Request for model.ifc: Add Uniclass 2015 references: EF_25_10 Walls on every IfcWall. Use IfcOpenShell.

First a look at what the model holds.

```python
import ifcopenshell

model = ifcopenshell.open("model.ifc")
print(model.schema)
print("classifications:", [c.Name for c in model.by_type("IfcClassification")])
for ifc_class in ("IfcDoor", "IfcRoof", "IfcStair", "IfcWall", "IfcWindow"):
    print(ifc_class, len(model.by_type(ifc_class)))
```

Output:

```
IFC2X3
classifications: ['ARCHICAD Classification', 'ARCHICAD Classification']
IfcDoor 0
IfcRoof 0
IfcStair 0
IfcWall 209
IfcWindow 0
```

```python
import ifcopenshell
import ifcopenshell.api.classification

model = ifcopenshell.open("model.ifc")

# IFC2X3 requires Source and Edition and has no link from the project to the system.
system = model.create_entity("IfcClassification", Source="NBS", Edition="2015", Name="Uniclass 2015")

codes = {
    "IfcWall": ("EF_25_10", "Walls"),
}
for ifc_class, (code, name) in codes.items():
    products = model.by_type(ifc_class)
    ifcopenshell.api.classification.add_reference(
        model, products=products, classification=system, identification=code, name=name
    )
    print(code, len(products))

model.write("model_rev.ifc")
```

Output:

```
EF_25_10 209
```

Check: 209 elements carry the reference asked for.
